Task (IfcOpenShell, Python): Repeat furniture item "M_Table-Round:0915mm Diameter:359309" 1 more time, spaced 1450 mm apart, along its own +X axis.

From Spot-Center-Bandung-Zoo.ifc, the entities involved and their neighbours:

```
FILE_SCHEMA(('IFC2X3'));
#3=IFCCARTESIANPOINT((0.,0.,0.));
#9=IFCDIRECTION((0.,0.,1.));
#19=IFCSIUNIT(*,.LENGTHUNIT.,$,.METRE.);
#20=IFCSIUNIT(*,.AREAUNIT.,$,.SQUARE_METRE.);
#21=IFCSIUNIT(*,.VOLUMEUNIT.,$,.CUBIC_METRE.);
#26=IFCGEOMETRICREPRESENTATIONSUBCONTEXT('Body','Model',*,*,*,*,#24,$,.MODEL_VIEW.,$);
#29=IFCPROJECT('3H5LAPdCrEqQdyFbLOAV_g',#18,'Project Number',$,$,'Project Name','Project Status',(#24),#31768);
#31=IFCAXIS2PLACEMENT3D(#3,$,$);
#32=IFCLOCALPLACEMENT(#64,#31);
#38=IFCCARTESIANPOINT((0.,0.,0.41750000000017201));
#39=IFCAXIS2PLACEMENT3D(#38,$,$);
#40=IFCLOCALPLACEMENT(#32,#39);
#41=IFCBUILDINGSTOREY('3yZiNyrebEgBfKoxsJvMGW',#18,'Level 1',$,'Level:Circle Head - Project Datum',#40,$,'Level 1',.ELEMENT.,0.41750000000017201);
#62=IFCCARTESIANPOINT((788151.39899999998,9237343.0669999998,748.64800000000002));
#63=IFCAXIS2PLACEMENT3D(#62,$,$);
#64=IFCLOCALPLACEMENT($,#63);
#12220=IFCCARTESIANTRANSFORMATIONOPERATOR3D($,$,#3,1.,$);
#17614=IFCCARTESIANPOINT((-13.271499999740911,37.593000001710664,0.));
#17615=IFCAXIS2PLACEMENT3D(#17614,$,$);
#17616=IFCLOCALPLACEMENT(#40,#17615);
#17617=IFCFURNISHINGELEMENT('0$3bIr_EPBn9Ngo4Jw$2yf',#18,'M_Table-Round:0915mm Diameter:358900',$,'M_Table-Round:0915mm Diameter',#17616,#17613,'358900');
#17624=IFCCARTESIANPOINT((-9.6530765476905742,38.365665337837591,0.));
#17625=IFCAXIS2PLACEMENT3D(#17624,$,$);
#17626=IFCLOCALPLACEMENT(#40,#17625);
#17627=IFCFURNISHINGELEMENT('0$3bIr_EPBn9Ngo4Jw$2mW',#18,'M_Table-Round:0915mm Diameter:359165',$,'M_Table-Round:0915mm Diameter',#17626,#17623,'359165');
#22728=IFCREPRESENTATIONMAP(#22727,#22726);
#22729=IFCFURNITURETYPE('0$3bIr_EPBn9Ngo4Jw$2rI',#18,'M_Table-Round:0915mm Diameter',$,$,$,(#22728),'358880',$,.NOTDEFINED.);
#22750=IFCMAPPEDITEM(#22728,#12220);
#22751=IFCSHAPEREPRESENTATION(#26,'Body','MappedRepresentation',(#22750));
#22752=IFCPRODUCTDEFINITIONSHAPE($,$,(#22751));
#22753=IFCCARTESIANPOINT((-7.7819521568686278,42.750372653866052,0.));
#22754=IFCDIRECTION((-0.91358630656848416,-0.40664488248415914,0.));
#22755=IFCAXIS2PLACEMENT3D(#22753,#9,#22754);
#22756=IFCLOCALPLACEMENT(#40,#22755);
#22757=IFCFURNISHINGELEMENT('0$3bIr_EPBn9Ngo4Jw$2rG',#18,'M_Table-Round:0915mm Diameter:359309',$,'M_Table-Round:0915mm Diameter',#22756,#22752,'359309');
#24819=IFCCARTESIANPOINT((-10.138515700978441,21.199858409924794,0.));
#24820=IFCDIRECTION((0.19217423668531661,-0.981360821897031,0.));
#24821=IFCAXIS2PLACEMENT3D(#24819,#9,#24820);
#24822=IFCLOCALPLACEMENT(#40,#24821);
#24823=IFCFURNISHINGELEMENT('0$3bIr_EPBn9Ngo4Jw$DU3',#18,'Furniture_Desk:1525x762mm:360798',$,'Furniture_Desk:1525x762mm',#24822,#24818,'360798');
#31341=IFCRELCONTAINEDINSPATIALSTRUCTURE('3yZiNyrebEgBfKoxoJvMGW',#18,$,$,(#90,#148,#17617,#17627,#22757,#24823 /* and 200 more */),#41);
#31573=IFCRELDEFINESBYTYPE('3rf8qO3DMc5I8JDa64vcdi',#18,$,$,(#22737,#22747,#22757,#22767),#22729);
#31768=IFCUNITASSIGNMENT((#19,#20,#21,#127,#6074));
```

```python
import ifcopenshell
import ifcopenshell.api.geometry
import ifcopenshell.api.root
import ifcopenshell.util.element
import ifcopenshell.util.placement

model = ifcopenshell.open("Spot-Center-Bandung-Zoo.ifc")


def reuse_history(source, copy):
    """copy_class also copies each property set's owner history, people and application; keep the originals."""
    for rel in copy.IsDefinedBy:
        if rel.is_a("IfcRelDefinesByProperties") and (history := rel.RelatingPropertyDefinition.OwnerHistory):
            rel.RelatingPropertyDefinition.OwnerHistory = source.OwnerHistory
            ifcopenshell.util.element.remove_deep2(model, history)


source = model.by_guid("0$3bIr_EPBn9Ngo4Jw$2rG")
base = ifcopenshell.util.placement.get_local_placement(source.ObjectPlacement)
step = base[:3, 0] * 1.45

for i in range(1, 2):
    copy = ifcopenshell.api.root.copy_class(model, product=source)
    copy.Representation = ifcopenshell.util.element.copy_deep(
        model, source.Representation, exclude=["IfcGeometricRepresentationContext", "IfcRepresentationMap"]
    )
    copy.Name = "M_Table-Round:0915mm Diameter"
    copy.Tag = None
    reuse_history(source, copy)
    matrix = base.copy()
    matrix[:3, 3] += i * step
    print("added at", matrix[:3, 3].round(3) + 0.0)
    ifcopenshell.api.geometry.edit_object_placement(model, product=copy, matrix=matrix, is_si=False)

model.write("Spot-Center-Bandung-Zoo_edited.ifc")
```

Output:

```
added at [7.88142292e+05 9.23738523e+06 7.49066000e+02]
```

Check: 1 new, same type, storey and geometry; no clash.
